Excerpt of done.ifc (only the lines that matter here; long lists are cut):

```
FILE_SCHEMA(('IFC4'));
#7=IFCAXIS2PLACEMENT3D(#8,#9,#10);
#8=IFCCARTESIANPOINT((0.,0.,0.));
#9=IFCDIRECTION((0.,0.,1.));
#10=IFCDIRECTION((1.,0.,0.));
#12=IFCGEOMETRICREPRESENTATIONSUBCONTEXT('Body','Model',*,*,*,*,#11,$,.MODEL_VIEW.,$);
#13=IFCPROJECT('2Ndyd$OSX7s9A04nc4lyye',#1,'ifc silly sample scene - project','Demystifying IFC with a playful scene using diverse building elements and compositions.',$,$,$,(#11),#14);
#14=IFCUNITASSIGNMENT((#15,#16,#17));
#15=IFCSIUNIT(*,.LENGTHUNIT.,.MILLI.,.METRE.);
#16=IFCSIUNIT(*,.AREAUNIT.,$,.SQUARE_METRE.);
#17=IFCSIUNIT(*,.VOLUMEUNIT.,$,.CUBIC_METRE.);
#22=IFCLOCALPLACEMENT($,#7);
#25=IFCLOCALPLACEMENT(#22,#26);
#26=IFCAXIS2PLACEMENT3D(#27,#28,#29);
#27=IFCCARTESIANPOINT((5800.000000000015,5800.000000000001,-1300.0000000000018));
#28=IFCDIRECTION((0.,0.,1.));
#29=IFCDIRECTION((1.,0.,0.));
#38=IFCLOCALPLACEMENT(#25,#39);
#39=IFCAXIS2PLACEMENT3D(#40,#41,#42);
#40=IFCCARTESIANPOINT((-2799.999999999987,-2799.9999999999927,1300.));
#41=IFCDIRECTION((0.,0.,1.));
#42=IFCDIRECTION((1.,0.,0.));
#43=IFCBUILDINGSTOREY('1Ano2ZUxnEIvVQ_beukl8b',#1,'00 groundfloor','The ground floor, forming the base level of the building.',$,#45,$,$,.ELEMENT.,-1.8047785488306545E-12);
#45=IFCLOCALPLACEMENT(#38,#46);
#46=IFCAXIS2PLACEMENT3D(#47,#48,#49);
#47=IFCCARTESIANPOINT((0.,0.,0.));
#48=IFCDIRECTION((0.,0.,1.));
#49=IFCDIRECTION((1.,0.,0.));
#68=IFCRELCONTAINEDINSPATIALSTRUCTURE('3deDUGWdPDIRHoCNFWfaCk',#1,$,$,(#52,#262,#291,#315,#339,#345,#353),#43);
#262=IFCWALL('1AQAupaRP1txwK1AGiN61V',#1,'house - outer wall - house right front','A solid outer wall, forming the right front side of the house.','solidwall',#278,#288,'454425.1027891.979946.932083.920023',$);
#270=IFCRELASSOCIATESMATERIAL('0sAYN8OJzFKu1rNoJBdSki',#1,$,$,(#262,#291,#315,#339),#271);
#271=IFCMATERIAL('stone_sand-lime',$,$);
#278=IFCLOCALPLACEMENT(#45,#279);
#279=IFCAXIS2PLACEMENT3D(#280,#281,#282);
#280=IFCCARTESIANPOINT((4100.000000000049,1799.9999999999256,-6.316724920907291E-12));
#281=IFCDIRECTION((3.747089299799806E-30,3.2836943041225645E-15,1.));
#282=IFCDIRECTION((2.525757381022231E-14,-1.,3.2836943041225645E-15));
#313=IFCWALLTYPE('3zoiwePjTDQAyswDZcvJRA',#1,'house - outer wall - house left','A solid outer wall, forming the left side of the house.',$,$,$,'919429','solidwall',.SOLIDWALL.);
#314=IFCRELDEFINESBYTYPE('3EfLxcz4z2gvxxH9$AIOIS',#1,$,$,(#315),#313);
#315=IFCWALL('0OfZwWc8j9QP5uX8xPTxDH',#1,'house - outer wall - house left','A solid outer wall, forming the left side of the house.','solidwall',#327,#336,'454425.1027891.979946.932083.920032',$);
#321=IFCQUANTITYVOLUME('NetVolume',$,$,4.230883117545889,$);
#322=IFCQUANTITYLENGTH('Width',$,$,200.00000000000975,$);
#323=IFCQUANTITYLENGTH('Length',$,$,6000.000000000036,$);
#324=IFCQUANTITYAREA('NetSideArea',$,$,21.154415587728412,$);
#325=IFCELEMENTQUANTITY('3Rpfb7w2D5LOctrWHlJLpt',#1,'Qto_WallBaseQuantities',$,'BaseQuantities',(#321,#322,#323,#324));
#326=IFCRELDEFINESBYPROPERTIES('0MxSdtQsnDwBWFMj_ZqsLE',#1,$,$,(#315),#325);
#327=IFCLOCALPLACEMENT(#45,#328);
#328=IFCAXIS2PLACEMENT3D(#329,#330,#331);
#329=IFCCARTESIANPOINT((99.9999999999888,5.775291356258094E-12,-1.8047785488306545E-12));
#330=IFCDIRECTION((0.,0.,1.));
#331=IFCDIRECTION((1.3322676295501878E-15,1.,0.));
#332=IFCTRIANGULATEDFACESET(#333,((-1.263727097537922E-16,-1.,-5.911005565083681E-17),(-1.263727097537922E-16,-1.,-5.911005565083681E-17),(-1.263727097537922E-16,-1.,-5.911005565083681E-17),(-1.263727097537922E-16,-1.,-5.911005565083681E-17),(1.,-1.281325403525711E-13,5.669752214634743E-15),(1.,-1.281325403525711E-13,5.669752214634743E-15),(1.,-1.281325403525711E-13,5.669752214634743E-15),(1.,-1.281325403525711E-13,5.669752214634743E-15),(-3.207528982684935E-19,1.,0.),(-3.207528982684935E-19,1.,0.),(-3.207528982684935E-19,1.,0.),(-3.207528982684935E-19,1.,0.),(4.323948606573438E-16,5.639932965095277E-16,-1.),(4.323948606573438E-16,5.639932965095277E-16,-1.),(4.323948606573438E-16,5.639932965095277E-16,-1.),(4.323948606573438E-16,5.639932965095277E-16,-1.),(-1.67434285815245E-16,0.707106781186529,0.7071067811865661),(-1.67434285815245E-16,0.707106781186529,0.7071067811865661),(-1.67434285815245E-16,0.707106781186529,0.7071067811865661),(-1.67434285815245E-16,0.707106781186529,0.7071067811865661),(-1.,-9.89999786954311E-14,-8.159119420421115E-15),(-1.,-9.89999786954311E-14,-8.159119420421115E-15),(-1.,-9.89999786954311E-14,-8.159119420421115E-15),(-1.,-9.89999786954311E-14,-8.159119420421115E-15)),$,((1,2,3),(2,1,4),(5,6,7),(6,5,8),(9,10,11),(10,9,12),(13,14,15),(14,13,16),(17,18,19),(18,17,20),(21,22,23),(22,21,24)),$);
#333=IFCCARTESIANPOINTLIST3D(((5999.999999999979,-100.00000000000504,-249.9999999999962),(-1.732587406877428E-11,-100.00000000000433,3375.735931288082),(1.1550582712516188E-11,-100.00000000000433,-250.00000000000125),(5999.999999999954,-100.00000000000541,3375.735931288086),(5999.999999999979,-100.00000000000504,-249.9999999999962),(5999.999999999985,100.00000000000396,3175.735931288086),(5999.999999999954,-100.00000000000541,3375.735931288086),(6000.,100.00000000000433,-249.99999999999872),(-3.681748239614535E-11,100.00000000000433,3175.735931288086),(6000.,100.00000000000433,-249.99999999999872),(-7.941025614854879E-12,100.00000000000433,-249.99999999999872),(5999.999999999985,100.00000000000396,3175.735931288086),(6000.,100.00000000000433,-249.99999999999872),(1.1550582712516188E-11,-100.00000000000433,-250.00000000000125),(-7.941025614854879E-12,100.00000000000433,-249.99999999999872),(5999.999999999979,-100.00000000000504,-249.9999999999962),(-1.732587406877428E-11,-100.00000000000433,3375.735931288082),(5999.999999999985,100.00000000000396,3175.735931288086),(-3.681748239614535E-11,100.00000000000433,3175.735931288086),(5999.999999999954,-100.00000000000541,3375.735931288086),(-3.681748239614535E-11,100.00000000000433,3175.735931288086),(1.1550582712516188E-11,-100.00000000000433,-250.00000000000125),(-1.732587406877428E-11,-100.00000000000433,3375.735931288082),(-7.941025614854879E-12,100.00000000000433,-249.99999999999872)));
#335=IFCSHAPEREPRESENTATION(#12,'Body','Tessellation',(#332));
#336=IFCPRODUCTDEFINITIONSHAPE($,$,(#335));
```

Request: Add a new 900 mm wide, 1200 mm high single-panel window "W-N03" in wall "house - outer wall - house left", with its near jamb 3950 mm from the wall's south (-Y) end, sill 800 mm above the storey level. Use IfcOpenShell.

```python
import numpy as np
import ifcopenshell
import ifcopenshell.api.feature
import ifcopenshell.api.geometry
import ifcopenshell.api.pset
import ifcopenshell.api.root
import ifcopenshell.api.spatial
import ifcopenshell.geom
import ifcopenshell.util.element
import ifcopenshell.util.placement
import ifcopenshell.util.representation
import ifcopenshell.util.shape
import ifcopenshell.util.unit

model = ifcopenshell.open("done.ifc")
unit_scale = ifcopenshell.util.unit.calculate_unit_scale(model)
area_scale = ifcopenshell.util.unit.calculate_unit_scale(model, "AREAUNIT")
volume_scale = ifcopenshell.util.unit.calculate_unit_scale(model, "VOLUMEUNIT")
settings = ifcopenshell.geom.settings()


def volume(element):
    """Net volume in cubic metres, openings subtracted."""
    shape = ifcopenshell.geom.create_shape(settings, element)
    return ifcopenshell.util.shape.get_volume(shape.geometry)


wall = model.by_guid("0OfZwWc8j9QP5uX8xPTxDH")
storey = ifcopenshell.util.element.get_container(wall, ifc_class="IfcBuildingStorey")
context = ifcopenshell.util.representation.get_context(model, "Model", "Body", "MODEL_VIEW")
before = volume(wall)

width, height, from_end, sill = 0.9, 1.2, 3.95, 0.8  # metres

# The wall runs along its own X axis, and the end named is its -X end.
wall_shape = ifcopenshell.geom.create_shape(settings, wall)
x, y, z = ifcopenshell.util.shape.get_vertices(wall_shape.geometry).T
start = x.min() + from_end
face, thickness = float(y.min()), float(y.max() - y.min())
wall_matrix = ifcopenshell.util.placement.get_local_placement(wall.ObjectPlacement)
level = ifcopenshell.util.placement.get_local_placement(storey.ObjectPlacement)[2, 3]


def in_wall(x, y):
    """Placement at x, y metres in the wall's axes, at sill height."""
    matrix = wall_matrix.copy()
    matrix[:, 3] = wall_matrix @ np.array([x / unit_scale, y / unit_scale, 0.0, 1.0])
    matrix[2, 3] = level + sill / unit_scale
    return matrix


# Opening: a box that overshoots both wall faces by 50 mm.
opening = ifcopenshell.api.root.create_entity(model, ifc_class="IfcOpeningElement", predefined_type="OPENING")
box = ifcopenshell.api.geometry.add_wall_representation(
    model, context=context, length=width, height=height, thickness=thickness + 0.1
)
ifcopenshell.api.geometry.assign_representation(model, product=opening, representation=box)
ifcopenshell.api.geometry.edit_object_placement(model, product=opening, matrix=in_wall(start, face - 0.05), is_si=False)
ifcopenshell.api.feature.add_feature(model, feature=opening, element=wall)

window = ifcopenshell.api.root.create_entity(model, ifc_class="IfcWindow", name="W-N03", predefined_type="WINDOW")
window.OverallWidth, window.OverallHeight = width / unit_scale, height / unit_scale
window.PartitioningType = "SINGLE_PANEL"
body = ifcopenshell.api.geometry.add_window_representation(
    model,
    context=context,
    overall_width=window.OverallWidth,
    overall_height=window.OverallHeight,
    partition_type="SINGLE_PANEL",
)
ifcopenshell.api.geometry.assign_representation(model, product=window, representation=body)
ifcopenshell.api.spatial.assign_container(model, products=[window], relating_structure=storey)
ifcopenshell.api.feature.add_filling(model, opening=opening, element=window)

# Centre the window in the wall's thickness.
ifcopenshell.api.geometry.edit_object_placement(model, product=window, matrix=in_wall(start, face), is_si=False)
window_shape = ifcopenshell.geom.create_shape(settings, window)
depth = ifcopenshell.util.shape.get_vertices(window_shape.geometry)[:, 1]
offset = face + thickness / 2 - (depth.min() + depth.max()) / 2
ifcopenshell.api.geometry.edit_object_placement(model, product=window, matrix=in_wall(start, offset), is_si=False)

after = volume(wall)

# Update the wall's stored quantities.
qto = model.by_id(ifcopenshell.util.element.get_pset(wall, "Qto_WallBaseQuantities", should_inherit=False)["id"])
ifcopenshell.api.pset.edit_qto(model, qto=qto, properties={
    "NetVolume": after / volume_scale,
    "NetSideArea": after / thickness / area_scale,
})

print(f"wall volume {before:.3f} -> {after:.3f} m3")

model.write("done-out.ifc")
```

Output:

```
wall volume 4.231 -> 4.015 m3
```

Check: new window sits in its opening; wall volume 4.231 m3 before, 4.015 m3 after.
